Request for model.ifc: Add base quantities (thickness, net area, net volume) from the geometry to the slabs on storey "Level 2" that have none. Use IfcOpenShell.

First a look at what the model holds.

```python
import ifcopenshell
import ifcopenshell.util.element
import ifcopenshell.util.unit

model = ifcopenshell.open("model.ifc")
print(model.schema)
for unit_type in ("LENGTHUNIT", "AREAUNIT", "VOLUMEUNIT"):
    print(unit_type, ifcopenshell.util.unit.calculate_unit_scale(model, unit_type))
storey = next(s for s in model.by_type("IfcBuildingStorey") if s.Name == "Level 2")
slabs = [e for e in ifcopenshell.util.element.get_decomposition(storey) if e.is_a("IfcSlab")]
for e in sorted(slabs, key=lambda e: e.id()):
    print(e.id(), e.is_a(), e.Name, list(ifcopenshell.util.element.get_psets(e, qtos_only=True)), sep=" | ")
```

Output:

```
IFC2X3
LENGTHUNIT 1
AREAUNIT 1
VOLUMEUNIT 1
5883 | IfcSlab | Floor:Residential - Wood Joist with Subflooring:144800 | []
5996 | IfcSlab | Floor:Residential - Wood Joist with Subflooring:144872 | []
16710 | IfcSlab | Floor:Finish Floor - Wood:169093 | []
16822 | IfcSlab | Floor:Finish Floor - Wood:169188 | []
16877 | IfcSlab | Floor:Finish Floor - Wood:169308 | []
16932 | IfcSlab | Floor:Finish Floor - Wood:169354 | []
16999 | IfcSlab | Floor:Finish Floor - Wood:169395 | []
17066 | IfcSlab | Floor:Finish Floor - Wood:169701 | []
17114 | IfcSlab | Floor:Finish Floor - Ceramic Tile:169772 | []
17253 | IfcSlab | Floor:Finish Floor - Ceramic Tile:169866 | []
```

```python
import ifcopenshell
import ifcopenshell.api.pset
import ifcopenshell.geom
import ifcopenshell.util.element
import ifcopenshell.util.shape
import ifcopenshell.util.unit

model = ifcopenshell.open("model.ifc")
unit_scale = ifcopenshell.util.unit.calculate_unit_scale(model)
area_scale = ifcopenshell.util.unit.calculate_unit_scale(model, "AREAUNIT")
volume_scale = ifcopenshell.util.unit.calculate_unit_scale(model, "VOLUMEUNIT")
settings = ifcopenshell.geom.settings()

storey = next(s for s in model.by_type("IfcBuildingStorey") if s.Name == "Level 2")
slabs = [e for e in ifcopenshell.util.element.get_decomposition(storey) if e.is_a("IfcSlab")]

for e in sorted(slabs, key=lambda e: e.id()):
    if ifcopenshell.util.element.get_psets(e, qtos_only=True, should_inherit=False):
        continue
    # Geometry comes back in metres, in the element's own axes.
    shape = ifcopenshell.geom.create_shape(settings, e)
    values = {
        "Width": ifcopenshell.util.shape.get_z(shape.geometry) / unit_scale,
        "NetArea": ifcopenshell.util.shape.get_footprint_area(shape.geometry) / area_scale,
        "NetVolume": ifcopenshell.util.shape.get_volume(shape.geometry) / volume_scale,
    }
    qto = ifcopenshell.api.pset.add_qto(model, product=e, name="BaseQuantities")
    ifcopenshell.api.pset.edit_qto(model, qto=qto, properties=values)
    print(e.id(), {k: round(v, 3) for k, v in values.items()})

model.write("model_v2.ifc")
```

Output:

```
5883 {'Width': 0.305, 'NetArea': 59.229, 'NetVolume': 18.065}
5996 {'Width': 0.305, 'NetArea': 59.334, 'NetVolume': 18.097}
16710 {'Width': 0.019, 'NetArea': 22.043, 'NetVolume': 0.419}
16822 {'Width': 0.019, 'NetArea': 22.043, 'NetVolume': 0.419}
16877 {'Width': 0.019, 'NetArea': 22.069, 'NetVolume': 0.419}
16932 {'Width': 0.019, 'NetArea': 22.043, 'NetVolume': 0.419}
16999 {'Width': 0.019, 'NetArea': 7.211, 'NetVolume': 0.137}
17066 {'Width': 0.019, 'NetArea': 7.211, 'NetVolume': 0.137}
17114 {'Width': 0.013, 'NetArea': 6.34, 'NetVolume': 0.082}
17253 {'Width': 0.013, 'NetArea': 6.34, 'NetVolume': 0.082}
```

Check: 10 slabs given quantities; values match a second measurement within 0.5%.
